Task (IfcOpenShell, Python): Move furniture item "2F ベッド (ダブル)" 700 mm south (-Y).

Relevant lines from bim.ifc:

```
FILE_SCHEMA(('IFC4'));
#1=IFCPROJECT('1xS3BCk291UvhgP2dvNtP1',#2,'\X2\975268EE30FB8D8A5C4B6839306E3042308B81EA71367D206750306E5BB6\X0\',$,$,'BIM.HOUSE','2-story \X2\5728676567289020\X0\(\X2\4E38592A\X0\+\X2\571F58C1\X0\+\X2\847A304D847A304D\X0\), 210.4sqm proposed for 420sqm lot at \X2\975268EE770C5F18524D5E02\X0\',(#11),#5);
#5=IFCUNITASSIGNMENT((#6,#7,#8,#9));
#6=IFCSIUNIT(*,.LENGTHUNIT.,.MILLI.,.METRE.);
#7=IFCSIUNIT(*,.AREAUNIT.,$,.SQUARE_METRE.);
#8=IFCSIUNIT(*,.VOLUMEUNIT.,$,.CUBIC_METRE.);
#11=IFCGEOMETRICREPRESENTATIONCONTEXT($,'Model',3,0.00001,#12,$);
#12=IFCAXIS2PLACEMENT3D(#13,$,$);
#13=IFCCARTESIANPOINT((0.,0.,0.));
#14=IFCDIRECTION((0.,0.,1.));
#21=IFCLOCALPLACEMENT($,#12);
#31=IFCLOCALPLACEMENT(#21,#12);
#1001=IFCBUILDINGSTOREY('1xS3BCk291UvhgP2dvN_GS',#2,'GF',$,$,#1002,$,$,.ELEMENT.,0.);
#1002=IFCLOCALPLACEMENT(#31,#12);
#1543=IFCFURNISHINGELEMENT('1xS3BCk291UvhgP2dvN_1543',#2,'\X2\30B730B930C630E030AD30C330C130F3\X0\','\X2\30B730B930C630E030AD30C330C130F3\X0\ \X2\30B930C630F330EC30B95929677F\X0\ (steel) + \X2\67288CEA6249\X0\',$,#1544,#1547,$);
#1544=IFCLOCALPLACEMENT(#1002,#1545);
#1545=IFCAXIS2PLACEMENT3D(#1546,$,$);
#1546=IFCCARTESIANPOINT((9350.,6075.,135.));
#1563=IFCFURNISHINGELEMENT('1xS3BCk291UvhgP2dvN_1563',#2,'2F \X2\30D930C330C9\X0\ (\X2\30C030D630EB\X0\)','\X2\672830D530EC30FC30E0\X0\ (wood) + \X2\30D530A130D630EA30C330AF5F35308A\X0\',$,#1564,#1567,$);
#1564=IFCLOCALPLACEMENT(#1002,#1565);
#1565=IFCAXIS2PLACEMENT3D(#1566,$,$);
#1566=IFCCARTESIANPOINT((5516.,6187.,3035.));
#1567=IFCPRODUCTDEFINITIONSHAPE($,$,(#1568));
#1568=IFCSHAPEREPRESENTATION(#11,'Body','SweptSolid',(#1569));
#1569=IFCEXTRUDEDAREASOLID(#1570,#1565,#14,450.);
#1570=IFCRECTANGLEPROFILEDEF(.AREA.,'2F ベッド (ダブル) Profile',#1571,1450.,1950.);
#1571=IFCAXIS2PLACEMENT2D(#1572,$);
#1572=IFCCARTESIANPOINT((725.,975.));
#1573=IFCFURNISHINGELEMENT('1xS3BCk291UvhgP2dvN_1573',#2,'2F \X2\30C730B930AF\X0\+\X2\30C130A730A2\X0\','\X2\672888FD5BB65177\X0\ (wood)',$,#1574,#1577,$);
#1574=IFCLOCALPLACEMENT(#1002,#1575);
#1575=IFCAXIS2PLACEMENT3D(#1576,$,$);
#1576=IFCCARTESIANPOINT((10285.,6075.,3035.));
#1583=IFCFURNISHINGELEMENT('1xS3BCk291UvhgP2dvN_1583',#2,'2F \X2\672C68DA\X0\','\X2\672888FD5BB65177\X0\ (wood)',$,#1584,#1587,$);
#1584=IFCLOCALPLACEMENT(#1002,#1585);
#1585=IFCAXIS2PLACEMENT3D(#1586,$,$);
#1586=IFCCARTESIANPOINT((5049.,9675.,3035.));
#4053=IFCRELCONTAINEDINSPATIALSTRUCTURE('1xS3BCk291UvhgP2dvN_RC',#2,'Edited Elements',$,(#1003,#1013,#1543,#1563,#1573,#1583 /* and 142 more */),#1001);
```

```python
import ifcopenshell
import ifcopenshell.api.geometry
import ifcopenshell.util.placement
import ifcopenshell.util.unit

model = ifcopenshell.open("bim.ifc")
unit_scale = ifcopenshell.util.unit.calculate_unit_scale(model)

item = model.by_id(1563)
matrix = ifcopenshell.util.placement.get_local_placement(item.ObjectPlacement)
matrix[1, 3] -= 0.7 / unit_scale
ifcopenshell.api.geometry.edit_object_placement(model, product=item, matrix=matrix, is_si=False)

print(ifcopenshell.util.placement.get_local_placement(item.ObjectPlacement).round(3) + 0.0)

model.write("bim_edited.ifc")
```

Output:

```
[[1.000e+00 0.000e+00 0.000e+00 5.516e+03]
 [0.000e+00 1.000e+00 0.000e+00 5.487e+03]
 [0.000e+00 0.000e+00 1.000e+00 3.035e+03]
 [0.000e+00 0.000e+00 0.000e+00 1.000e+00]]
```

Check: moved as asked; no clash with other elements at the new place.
